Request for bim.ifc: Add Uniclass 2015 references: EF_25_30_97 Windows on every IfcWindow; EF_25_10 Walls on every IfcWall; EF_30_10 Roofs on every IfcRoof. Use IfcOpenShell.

First a look at what the model holds.

```python
import ifcopenshell

model = ifcopenshell.open("bim.ifc")
print(model.schema)
print("classifications:", [c.Name for c in model.by_type("IfcClassification")])
for ifc_class in ("IfcDoor", "IfcRoof", "IfcStair", "IfcWall", "IfcWindow"):
    print(ifc_class, len(model.by_type(ifc_class)))
```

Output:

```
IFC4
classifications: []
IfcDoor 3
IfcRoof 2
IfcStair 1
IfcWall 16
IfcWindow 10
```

```python
import ifcopenshell
import ifcopenshell.api.classification

model = ifcopenshell.open("bim.ifc")

system = ifcopenshell.api.classification.add_classification(model, classification="Uniclass 2015")

codes = {
    "IfcWindow": ("EF_25_30_97", "Windows"),
    "IfcWall": ("EF_25_10", "Walls"),
    "IfcRoof": ("EF_30_10", "Roofs"),
}
for ifc_class, (code, name) in codes.items():
    products = model.by_type(ifc_class)
    ifcopenshell.api.classification.add_reference(
        model, products=products, classification=system, identification=code, name=name
    )
    print(code, len(products))

model.write("bim_rev.ifc")
```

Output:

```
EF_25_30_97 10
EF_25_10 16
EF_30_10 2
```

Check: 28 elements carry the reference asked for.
